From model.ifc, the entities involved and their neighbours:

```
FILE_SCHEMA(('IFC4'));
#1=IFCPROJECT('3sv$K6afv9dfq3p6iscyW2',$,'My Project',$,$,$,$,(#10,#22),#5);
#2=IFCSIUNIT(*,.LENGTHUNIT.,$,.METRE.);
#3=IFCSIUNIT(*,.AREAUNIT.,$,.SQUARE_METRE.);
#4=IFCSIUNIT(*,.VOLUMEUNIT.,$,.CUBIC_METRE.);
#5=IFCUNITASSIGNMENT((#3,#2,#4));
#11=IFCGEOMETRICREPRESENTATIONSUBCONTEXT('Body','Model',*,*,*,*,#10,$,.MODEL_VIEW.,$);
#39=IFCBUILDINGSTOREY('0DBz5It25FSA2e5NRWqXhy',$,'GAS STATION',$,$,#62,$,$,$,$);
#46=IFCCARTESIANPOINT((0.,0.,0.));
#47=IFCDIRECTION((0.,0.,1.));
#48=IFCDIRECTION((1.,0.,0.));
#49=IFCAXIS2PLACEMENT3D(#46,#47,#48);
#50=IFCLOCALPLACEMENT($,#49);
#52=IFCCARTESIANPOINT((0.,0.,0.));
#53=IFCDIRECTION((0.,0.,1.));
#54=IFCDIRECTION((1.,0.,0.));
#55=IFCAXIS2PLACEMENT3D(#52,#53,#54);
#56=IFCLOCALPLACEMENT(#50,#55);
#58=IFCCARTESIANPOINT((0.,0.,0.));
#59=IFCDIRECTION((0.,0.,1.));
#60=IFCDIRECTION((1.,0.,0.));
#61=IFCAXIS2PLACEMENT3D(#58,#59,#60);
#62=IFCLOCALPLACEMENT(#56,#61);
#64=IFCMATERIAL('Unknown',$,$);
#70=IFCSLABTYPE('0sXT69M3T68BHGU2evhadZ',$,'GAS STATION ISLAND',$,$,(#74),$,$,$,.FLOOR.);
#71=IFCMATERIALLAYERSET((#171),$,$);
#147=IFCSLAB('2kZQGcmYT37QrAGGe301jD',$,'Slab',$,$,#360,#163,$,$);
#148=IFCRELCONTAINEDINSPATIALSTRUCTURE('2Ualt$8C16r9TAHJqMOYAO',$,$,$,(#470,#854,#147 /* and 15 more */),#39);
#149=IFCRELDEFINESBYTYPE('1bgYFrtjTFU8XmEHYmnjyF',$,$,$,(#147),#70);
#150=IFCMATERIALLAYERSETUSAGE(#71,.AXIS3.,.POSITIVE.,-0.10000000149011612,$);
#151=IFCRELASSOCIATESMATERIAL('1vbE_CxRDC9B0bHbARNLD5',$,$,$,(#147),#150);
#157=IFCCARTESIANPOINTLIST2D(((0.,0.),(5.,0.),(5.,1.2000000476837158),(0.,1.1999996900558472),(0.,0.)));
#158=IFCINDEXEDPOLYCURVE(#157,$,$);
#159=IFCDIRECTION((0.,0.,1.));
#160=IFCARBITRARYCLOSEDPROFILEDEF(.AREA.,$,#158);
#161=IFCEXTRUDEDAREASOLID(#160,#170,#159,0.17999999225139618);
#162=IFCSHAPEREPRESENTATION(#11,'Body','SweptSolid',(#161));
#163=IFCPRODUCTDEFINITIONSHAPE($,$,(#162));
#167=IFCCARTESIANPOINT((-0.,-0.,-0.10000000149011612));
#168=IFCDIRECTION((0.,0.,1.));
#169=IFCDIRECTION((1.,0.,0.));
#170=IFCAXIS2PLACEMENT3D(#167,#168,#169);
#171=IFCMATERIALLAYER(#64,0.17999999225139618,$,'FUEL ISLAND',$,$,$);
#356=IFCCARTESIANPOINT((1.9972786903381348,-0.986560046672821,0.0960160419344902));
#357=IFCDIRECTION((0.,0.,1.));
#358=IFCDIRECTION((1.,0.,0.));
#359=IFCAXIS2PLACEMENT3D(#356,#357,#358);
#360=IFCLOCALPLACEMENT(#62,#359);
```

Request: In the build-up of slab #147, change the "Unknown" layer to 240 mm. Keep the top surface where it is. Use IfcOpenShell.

```python
import ifcopenshell
import ifcopenshell.util.element
import ifcopenshell.util.representation
import ifcopenshell.util.unit

model = ifcopenshell.open("model.ifc")
unit_scale = ifcopenshell.util.unit.calculate_unit_scale(model)

layer_set = model.by_id(71)
layer = next(l for l in layer_set.MaterialLayers if l.Material and l.Material.Name == "Unknown")
change = 0.24 / unit_scale - layer.LayerThickness
layer.LayerThickness += change

# Geometry does not follow the layer set by itself.
slabs = [e for e in ifcopenshell.util.element.get_elements_by_material(model, layer_set) if e.is_a("IfcSlab")]
for slab in sorted(slabs, key=lambda e: e.id()):
    body = ifcopenshell.util.representation.get_representation(slab, "Model", "Body")
    solid = body.Items[0]
    old_depth = solid.Depth
    solid.Depth += change
    # Extruded upwards: lower the start of the extrusion so the top stays.
    x, y, z = solid.Position.Location.Coordinates
    solid.Position.Location = model.createIfcCartesianPoint((x, y, z - change))
    print(slab.id(), f"{old_depth:g} -> {solid.Depth:g}")

# The layers are counted up from the underside, which has moved.
for usage in {ifcopenshell.util.element.get_material(slab) for slab in slabs}:
    usage.OffsetFromReferenceLine -= change

model.write("model-out.ifc")
```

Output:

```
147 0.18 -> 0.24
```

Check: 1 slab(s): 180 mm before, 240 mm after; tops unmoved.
